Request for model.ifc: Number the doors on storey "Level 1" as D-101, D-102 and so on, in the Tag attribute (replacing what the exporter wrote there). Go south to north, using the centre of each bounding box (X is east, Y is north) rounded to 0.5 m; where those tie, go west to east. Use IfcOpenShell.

First a look at what the model holds.

```python
import ifcopenshell
import ifcopenshell.util.element
import ifcopenshell.util.placement

model = ifcopenshell.open("model.ifc")
print(model.schema)
storey = next(s for s in model.by_type("IfcBuildingStorey") if s.Name == "Level 1")
doors = [e for e in ifcopenshell.util.element.get_decomposition(storey) if e.is_a("IfcDoor")]
for e in sorted(doors, key=lambda e: e.id()):
    origin = ifcopenshell.util.placement.get_local_placement(e.ObjectPlacement)[:3, 3]
    print(e.id(), e.Tag, e.Name, origin.round(2) + 0.0, sep=" | ")
```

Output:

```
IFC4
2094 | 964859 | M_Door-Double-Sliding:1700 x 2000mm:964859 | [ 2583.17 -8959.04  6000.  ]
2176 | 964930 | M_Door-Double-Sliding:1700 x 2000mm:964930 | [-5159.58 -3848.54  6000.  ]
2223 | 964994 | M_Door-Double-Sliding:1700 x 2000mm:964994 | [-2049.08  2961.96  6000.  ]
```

```python
import ifcopenshell
import ifcopenshell.geom
import ifcopenshell.util.element
import ifcopenshell.util.shape

model = ifcopenshell.open("model.ifc")
settings = ifcopenshell.geom.settings()
settings.set("use-world-coords", True)


def centre(element):
    shape = ifcopenshell.geom.create_shape(settings, element)
    return ifcopenshell.util.shape.get_bbox_centroid(shape.geometry)


storey = next(s for s in model.by_type("IfcBuildingStorey") if s.Name == "Level 1")
doors = [e for e in ifcopenshell.util.element.get_decomposition(storey) if e.is_a("IfcDoor")]

# Insertion points can sit at a corner or the storey origin, so sort by the geometry (in metres).
centres = {e: centre(e) for e in doors}
doors.sort(key=lambda e: (round(centres[e][1] / 0.5), centres[e][0]))

for i, e in enumerate(doors, start=1):
    number = f"D-1{i:02d}"
    e.Tag = number
    print(e.id(), number)

model.write("model_updated.ifc")
```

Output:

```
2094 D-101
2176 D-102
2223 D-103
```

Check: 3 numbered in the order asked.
